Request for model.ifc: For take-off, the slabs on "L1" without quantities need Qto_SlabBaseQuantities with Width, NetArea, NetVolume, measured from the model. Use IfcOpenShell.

First a look at what the model holds.

```python
import ifcopenshell
import ifcopenshell.util.element
import ifcopenshell.util.unit

model = ifcopenshell.open("model.ifc")
print(model.schema)
for unit_type in ("LENGTHUNIT", "AREAUNIT", "VOLUMEUNIT"):
    print(unit_type, ifcopenshell.util.unit.calculate_unit_scale(model, unit_type))
storey = next(s for s in model.by_type("IfcBuildingStorey") if s.Name == "L1")
slabs = [e for e in ifcopenshell.util.element.get_decomposition(storey) if e.is_a("IfcSlab")]
for e in sorted(slabs, key=lambda e: e.id()):
    print(e.id(), e.is_a(), e.Name, list(ifcopenshell.util.element.get_psets(e, qtos_only=True)), sep=" | ")
```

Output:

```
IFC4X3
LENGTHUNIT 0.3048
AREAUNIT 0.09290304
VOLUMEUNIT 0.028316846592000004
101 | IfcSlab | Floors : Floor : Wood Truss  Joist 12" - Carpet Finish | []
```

```python
import ifcopenshell
import ifcopenshell.api.pset
import ifcopenshell.geom
import ifcopenshell.util.element
import ifcopenshell.util.shape
import ifcopenshell.util.unit

model = ifcopenshell.open("model.ifc")
unit_scale = ifcopenshell.util.unit.calculate_unit_scale(model)
area_scale = ifcopenshell.util.unit.calculate_unit_scale(model, "AREAUNIT")
volume_scale = ifcopenshell.util.unit.calculate_unit_scale(model, "VOLUMEUNIT")
settings = ifcopenshell.geom.settings()

storey = next(s for s in model.by_type("IfcBuildingStorey") if s.Name == "L1")
slabs = [e for e in ifcopenshell.util.element.get_decomposition(storey) if e.is_a("IfcSlab")]

for e in sorted(slabs, key=lambda e: e.id()):
    if ifcopenshell.util.element.get_psets(e, qtos_only=True, should_inherit=False):
        continue
    # Geometry comes back in metres, in the element's own axes.
    shape = ifcopenshell.geom.create_shape(settings, e)
    values = {
        "Width": ifcopenshell.util.shape.get_z(shape.geometry) / unit_scale,
        "NetArea": ifcopenshell.util.shape.get_footprint_area(shape.geometry) / area_scale,
        "NetVolume": ifcopenshell.util.shape.get_volume(shape.geometry) / volume_scale,
    }
    qto = ifcopenshell.api.pset.add_qto(model, product=e, name="Qto_SlabBaseQuantities")
    ifcopenshell.api.pset.edit_qto(model, qto=qto, properties=values)
    print(e.id(), {k: round(v, 3) for k, v in values.items()})

model.write("model_edited.ifc")
```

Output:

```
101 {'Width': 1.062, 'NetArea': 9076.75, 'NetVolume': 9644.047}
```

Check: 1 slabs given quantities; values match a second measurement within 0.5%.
